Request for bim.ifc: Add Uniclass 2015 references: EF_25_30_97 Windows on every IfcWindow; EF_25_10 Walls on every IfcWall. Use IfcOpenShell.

First a look at what the model holds.

```python
import ifcopenshell

model = ifcopenshell.open("bim.ifc")
print(model.schema)
print("classifications:", [c.Name for c in model.by_type("IfcClassification")])
for ifc_class in ("IfcDoor", "IfcRoof", "IfcStair", "IfcWall", "IfcWindow"):
    print(ifc_class, len(model.by_type(ifc_class)))
```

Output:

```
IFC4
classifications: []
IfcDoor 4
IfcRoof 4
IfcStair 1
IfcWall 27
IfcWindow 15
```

```python
import ifcopenshell
import ifcopenshell.api.classification

model = ifcopenshell.open("bim.ifc")

system = ifcopenshell.api.classification.add_classification(model, classification="Uniclass 2015")

codes = {
    "IfcWindow": ("EF_25_30_97", "Windows"),
    "IfcWall": ("EF_25_10", "Walls"),
}
for ifc_class, (code, name) in codes.items():
    products = model.by_type(ifc_class)
    ifcopenshell.api.classification.add_reference(
        model, products=products, classification=system, identification=code, name=name
    )
    print(code, len(products))

model.write("bim_edited.ifc")
```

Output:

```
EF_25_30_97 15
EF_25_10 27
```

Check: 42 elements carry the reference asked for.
